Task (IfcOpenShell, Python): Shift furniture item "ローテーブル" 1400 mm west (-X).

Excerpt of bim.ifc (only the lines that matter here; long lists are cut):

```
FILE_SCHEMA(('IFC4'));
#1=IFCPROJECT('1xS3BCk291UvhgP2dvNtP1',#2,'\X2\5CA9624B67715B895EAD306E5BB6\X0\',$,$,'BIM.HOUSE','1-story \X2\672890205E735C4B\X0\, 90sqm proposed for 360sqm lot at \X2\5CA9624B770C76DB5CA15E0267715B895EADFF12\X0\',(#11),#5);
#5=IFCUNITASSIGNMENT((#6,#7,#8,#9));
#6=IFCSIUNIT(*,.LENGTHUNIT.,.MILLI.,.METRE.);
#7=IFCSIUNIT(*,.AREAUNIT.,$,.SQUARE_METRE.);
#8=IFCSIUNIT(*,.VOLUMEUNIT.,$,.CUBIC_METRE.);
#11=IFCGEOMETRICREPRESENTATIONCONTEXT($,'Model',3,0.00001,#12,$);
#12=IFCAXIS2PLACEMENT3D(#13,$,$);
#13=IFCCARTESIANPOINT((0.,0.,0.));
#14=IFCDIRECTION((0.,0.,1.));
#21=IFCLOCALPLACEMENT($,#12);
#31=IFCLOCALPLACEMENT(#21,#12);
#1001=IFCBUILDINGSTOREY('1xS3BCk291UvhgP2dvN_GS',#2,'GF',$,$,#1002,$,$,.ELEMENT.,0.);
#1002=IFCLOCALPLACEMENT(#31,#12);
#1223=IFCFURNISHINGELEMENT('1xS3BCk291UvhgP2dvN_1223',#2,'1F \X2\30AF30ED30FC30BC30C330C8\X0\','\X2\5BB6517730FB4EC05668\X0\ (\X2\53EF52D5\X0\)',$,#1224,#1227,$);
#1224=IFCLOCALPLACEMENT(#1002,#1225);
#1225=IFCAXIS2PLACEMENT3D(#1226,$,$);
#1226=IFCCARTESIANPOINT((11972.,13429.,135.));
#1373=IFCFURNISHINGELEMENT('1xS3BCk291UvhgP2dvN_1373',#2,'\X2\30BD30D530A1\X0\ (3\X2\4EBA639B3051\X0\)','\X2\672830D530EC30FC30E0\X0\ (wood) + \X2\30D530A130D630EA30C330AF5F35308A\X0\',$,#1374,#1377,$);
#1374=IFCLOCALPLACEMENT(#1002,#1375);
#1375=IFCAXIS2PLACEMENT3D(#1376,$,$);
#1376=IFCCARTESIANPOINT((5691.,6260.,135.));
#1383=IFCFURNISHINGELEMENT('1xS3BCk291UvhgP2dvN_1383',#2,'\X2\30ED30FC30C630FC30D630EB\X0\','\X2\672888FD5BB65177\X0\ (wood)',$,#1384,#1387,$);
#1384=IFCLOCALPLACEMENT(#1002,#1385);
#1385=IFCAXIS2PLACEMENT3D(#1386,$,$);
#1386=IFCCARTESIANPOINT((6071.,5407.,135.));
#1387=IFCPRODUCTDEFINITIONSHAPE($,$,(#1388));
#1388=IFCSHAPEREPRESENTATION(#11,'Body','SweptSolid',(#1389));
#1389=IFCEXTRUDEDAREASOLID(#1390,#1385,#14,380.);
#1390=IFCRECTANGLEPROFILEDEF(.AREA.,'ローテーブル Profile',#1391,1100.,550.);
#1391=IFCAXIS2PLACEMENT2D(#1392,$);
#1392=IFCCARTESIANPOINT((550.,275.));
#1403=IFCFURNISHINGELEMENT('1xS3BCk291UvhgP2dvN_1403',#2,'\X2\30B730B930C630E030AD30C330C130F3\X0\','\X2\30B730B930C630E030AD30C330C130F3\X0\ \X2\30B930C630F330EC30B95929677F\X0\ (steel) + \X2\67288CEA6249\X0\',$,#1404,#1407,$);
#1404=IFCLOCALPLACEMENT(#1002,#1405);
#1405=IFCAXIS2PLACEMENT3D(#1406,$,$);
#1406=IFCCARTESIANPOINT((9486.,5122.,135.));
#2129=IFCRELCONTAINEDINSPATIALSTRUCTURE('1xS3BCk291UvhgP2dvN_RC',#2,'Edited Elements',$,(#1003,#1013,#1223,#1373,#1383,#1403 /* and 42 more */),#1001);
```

```python
import ifcopenshell
import ifcopenshell.api.geometry
import ifcopenshell.util.placement
import ifcopenshell.util.unit

model = ifcopenshell.open("bim.ifc")
unit_scale = ifcopenshell.util.unit.calculate_unit_scale(model)

item = model.by_id(1383)
matrix = ifcopenshell.util.placement.get_local_placement(item.ObjectPlacement)
matrix[0, 3] -= 1.4 / unit_scale
ifcopenshell.api.geometry.edit_object_placement(model, product=item, matrix=matrix, is_si=False)

print(ifcopenshell.util.placement.get_local_placement(item.ObjectPlacement).round(3) + 0.0)

model.write("bim_updated.ifc")
```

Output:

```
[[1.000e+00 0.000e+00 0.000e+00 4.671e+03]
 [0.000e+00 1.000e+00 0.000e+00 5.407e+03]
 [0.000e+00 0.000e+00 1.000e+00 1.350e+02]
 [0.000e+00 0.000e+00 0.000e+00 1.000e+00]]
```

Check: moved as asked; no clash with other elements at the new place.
